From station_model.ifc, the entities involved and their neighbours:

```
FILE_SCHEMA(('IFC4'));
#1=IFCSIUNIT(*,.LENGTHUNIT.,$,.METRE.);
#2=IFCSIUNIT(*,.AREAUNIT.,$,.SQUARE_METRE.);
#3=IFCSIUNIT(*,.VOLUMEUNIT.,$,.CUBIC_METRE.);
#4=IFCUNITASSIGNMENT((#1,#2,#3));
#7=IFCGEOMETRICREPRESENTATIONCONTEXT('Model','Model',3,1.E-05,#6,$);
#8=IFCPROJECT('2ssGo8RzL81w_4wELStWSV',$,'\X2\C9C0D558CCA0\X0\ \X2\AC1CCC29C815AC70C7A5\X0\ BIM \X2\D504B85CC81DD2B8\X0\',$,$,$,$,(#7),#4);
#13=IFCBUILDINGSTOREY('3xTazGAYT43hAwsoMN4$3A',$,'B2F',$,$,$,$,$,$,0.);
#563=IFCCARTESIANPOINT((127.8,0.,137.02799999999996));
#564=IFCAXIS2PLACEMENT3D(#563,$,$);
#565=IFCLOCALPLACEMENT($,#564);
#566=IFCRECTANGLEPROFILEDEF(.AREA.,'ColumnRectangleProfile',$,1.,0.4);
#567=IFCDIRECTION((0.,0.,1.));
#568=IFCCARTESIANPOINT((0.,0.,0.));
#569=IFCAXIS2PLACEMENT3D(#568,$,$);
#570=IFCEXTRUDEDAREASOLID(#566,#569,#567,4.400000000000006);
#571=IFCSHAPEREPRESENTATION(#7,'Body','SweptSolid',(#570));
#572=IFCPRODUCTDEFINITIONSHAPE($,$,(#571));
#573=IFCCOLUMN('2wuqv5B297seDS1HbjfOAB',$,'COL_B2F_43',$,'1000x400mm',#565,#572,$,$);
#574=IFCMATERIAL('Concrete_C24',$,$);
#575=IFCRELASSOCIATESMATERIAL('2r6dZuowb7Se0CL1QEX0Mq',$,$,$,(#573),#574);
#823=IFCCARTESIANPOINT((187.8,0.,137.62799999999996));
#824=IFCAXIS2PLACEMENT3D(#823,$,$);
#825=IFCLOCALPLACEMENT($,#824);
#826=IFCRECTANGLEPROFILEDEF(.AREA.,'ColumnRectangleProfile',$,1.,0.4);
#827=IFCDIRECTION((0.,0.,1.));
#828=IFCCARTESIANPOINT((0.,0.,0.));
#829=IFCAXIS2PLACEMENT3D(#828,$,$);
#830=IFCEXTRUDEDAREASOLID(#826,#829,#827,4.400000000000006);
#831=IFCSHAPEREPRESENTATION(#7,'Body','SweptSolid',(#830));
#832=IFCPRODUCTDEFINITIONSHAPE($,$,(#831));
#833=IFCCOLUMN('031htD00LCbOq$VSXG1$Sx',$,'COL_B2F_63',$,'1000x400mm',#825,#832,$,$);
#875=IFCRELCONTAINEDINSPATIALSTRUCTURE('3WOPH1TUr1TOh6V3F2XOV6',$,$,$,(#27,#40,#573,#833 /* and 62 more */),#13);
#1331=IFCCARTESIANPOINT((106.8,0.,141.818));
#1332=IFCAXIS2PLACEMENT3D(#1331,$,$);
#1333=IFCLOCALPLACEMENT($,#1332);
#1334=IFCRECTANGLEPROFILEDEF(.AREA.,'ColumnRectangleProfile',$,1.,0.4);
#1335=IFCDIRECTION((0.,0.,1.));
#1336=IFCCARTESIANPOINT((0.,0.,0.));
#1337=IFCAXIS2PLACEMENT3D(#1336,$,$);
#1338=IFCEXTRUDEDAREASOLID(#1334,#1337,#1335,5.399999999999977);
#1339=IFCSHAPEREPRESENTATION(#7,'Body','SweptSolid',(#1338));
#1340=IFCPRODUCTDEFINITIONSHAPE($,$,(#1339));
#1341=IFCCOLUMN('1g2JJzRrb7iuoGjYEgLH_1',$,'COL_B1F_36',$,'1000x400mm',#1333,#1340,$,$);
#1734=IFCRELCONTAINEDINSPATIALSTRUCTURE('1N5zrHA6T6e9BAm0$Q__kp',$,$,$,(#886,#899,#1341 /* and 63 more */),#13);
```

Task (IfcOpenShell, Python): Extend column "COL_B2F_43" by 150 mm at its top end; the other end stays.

```python
import ifcopenshell

model = ifcopenshell.open("station_model.ifc")

member = model.by_guid("2wuqv5B297seDS1HbjfOAB")
change = 0.15

# The extrusion runs towards the end named, so only its depth changes.
body = next(r for r in member.Representation.Representations if r.RepresentationIdentifier == "Body")
solid = body.Items[0]
old_length = solid.Depth
solid.Depth += change

print(f"length {old_length:g} -> {solid.Depth:g}")

model.write("station_model_rev.ifc")
```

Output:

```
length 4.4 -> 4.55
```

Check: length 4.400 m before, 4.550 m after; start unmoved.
